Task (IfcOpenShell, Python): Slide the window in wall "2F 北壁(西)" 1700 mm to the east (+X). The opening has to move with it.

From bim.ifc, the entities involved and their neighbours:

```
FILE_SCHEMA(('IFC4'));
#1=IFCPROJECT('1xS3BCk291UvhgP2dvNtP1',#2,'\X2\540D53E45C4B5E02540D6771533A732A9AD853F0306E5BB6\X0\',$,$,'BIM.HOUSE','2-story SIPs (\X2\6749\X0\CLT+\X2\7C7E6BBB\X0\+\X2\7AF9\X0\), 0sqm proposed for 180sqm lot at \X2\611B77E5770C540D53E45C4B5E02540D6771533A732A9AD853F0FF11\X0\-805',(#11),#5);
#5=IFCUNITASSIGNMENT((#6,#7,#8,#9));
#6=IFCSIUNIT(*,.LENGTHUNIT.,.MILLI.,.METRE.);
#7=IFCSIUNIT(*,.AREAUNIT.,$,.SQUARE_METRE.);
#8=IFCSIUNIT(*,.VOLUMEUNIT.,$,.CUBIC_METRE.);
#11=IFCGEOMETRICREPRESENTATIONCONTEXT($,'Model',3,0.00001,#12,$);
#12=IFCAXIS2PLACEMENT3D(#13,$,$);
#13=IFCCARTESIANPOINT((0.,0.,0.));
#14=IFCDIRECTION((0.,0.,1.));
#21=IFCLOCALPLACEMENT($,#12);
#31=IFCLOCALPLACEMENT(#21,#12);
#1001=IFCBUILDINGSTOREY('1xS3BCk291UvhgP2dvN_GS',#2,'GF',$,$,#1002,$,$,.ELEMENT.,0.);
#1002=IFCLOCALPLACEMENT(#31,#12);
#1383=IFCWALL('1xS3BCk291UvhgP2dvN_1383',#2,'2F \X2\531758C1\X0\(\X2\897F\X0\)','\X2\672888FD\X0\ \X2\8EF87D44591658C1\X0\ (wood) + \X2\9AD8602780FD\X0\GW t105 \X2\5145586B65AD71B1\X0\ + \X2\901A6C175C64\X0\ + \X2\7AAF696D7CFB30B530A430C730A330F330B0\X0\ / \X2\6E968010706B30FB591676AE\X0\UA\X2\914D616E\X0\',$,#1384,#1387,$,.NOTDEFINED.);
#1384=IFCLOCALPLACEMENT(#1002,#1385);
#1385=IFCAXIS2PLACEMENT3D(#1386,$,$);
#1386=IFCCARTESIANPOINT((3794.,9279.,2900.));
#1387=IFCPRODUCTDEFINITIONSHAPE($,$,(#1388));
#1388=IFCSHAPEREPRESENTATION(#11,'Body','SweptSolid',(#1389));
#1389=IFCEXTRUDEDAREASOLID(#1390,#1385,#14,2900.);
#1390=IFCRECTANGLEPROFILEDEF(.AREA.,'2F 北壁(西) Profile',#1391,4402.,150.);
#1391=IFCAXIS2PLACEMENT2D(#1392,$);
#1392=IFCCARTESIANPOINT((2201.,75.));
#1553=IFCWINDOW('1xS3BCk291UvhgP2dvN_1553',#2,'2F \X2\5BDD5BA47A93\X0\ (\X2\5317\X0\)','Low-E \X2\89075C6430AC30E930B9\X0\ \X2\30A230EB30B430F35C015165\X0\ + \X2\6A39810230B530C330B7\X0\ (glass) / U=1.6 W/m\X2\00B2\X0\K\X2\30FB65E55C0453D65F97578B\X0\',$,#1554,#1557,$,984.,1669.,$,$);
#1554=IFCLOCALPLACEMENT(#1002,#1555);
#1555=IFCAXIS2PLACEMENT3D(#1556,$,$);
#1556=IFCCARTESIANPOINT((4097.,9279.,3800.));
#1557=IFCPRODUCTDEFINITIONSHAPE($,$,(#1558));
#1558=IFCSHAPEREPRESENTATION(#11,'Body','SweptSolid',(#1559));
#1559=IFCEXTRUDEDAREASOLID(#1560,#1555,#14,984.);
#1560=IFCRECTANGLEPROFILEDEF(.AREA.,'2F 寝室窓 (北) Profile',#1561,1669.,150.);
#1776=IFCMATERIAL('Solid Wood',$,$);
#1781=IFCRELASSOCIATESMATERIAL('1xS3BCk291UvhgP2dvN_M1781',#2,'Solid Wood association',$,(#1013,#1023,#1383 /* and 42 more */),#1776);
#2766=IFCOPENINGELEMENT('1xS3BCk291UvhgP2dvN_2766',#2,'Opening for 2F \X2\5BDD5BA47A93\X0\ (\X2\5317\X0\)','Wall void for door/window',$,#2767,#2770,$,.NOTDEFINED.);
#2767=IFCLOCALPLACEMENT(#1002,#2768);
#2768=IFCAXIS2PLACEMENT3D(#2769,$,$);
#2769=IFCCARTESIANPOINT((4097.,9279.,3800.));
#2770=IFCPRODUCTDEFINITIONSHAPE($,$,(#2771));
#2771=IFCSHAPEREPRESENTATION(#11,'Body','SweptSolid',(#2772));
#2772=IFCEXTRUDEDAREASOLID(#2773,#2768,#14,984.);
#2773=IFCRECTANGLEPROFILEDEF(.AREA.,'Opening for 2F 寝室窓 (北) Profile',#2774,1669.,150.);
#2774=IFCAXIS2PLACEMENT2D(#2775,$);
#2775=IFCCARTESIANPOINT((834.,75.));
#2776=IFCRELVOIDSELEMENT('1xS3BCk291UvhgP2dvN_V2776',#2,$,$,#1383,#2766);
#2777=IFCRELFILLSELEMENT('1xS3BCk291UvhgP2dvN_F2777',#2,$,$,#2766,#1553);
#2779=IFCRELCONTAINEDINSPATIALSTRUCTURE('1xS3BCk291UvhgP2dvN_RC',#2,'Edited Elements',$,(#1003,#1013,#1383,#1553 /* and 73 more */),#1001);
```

```python
import ifcopenshell
import ifcopenshell.api.geometry
import ifcopenshell.util.placement

model = ifcopenshell.open("bim.ifc")

window = model.by_id(1553)
opening = window.FillsVoids[0].RelatingOpeningElement
wall = opening.VoidsElements[0].RelatingBuildingElement

wall_matrix = ifcopenshell.util.placement.get_local_placement(wall.ObjectPlacement)
shift = wall_matrix[:3, 0] * 1700.0
before = ifcopenshell.util.placement.get_local_placement(window.ObjectPlacement)[:3, 3].copy()

# The window is not placed relative to its opening, so move both.
for product in (opening, window):
    matrix = ifcopenshell.util.placement.get_local_placement(product.ObjectPlacement)
    matrix[:3, 3] += shift
    ifcopenshell.api.geometry.edit_object_placement(model, product=product, matrix=matrix, is_si=False)

after = ifcopenshell.util.placement.get_local_placement(window.ObjectPlacement)[:3, 3]
print("window moved by", (after - before).round(3) + 0.0)

model.write("bim_updated.ifc")
```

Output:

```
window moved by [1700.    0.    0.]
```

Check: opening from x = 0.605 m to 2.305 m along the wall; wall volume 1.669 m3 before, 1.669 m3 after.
